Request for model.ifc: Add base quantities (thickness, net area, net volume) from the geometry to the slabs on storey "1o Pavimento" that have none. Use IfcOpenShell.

First a look at what the model holds.

```python
import ifcopenshell
import ifcopenshell.util.element
import ifcopenshell.util.unit

model = ifcopenshell.open("model.ifc")
print(model.schema)
for unit_type in ("LENGTHUNIT", "AREAUNIT", "VOLUMEUNIT"):
    print(unit_type, ifcopenshell.util.unit.calculate_unit_scale(model, unit_type))
storey = next(s for s in model.by_type("IfcBuildingStorey") if s.Name == "1o Pavimento")
slabs = [e for e in ifcopenshell.util.element.get_decomposition(storey) if e.is_a("IfcSlab")]
for e in sorted(slabs, key=lambda e: e.id()):
    print(e.id(), e.is_a(), e.Name, list(ifcopenshell.util.element.get_psets(e, qtos_only=True)), sep=" | ")
```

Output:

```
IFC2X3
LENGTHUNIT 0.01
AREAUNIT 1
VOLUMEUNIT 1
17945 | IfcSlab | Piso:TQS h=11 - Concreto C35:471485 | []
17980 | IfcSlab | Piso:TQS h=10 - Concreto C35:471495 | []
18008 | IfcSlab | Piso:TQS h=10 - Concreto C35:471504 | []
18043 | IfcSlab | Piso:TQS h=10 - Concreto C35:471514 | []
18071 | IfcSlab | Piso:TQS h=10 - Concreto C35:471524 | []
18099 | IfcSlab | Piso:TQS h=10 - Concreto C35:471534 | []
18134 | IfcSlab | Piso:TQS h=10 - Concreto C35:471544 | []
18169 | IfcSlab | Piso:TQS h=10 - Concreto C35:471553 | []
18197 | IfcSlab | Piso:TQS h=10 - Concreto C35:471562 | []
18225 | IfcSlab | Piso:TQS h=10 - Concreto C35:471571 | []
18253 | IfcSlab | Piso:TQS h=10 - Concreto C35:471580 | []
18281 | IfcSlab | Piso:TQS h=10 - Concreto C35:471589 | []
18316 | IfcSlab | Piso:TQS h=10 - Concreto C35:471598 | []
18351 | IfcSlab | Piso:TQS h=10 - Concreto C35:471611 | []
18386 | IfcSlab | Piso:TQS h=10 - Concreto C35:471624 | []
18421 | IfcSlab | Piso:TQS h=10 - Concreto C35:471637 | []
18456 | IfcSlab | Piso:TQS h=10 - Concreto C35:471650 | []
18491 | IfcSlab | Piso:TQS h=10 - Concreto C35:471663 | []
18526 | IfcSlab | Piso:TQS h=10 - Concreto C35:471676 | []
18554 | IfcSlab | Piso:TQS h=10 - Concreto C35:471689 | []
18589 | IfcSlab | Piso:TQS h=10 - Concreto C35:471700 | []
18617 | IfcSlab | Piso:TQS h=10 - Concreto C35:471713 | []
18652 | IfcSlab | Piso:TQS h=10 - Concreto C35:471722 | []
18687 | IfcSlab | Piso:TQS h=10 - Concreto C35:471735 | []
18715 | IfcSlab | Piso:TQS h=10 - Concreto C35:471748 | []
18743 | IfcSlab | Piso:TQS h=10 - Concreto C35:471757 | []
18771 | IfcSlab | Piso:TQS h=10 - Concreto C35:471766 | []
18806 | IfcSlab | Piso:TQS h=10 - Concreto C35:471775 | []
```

```python
import ifcopenshell
import ifcopenshell.api.pset
import ifcopenshell.geom
import ifcopenshell.util.element
import ifcopenshell.util.shape
import ifcopenshell.util.unit

model = ifcopenshell.open("model.ifc")
unit_scale = ifcopenshell.util.unit.calculate_unit_scale(model)
area_scale = ifcopenshell.util.unit.calculate_unit_scale(model, "AREAUNIT")
volume_scale = ifcopenshell.util.unit.calculate_unit_scale(model, "VOLUMEUNIT")
settings = ifcopenshell.geom.settings()

storey = next(s for s in model.by_type("IfcBuildingStorey") if s.Name == "1o Pavimento")
slabs = [e for e in ifcopenshell.util.element.get_decomposition(storey) if e.is_a("IfcSlab")]

for e in sorted(slabs, key=lambda e: e.id()):
    if ifcopenshell.util.element.get_psets(e, qtos_only=True, should_inherit=False):
        continue
    # Geometry comes back in metres, in the element's own axes.
    shape = ifcopenshell.geom.create_shape(settings, e)
    values = {
        "Width": ifcopenshell.util.shape.get_z(shape.geometry) / unit_scale,
        "NetArea": ifcopenshell.util.shape.get_footprint_area(shape.geometry) / area_scale,
        "NetVolume": ifcopenshell.util.shape.get_volume(shape.geometry) / volume_scale,
    }
    qto = ifcopenshell.api.pset.add_qto(model, product=e, name="BaseQuantities")
    ifcopenshell.api.pset.edit_qto(model, qto=qto, properties=values)
    print(e.id(), {k: round(v, 3) for k, v in values.items()})

model.write("model_v2.ifc")
```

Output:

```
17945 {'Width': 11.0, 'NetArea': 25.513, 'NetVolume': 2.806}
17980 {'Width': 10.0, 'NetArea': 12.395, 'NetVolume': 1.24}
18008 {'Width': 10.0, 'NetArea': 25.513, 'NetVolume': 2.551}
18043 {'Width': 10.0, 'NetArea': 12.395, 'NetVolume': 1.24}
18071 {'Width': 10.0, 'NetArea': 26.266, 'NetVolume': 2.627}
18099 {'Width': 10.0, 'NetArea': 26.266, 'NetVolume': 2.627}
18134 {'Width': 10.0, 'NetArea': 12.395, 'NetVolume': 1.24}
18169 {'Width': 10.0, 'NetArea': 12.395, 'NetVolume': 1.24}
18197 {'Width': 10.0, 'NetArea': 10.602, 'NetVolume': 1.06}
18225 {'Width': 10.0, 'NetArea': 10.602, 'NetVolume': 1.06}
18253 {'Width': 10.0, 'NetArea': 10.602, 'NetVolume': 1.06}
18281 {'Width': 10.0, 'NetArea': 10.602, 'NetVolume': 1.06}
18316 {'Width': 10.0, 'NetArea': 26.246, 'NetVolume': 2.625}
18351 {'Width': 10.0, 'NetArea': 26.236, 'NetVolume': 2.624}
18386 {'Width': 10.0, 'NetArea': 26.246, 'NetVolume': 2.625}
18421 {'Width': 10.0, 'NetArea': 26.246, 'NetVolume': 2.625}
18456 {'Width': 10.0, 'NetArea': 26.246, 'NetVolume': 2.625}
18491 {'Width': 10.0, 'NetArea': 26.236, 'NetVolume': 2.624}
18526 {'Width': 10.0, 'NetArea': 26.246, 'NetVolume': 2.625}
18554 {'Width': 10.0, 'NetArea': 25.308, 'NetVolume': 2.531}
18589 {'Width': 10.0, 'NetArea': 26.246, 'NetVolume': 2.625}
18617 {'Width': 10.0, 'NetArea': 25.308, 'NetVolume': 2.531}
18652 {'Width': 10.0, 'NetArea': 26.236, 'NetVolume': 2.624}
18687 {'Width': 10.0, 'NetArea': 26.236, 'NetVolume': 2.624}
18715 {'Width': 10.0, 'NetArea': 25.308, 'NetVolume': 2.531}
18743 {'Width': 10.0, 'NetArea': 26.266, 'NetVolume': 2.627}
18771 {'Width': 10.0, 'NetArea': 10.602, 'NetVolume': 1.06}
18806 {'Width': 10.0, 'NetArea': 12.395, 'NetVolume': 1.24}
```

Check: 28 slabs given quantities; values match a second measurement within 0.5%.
